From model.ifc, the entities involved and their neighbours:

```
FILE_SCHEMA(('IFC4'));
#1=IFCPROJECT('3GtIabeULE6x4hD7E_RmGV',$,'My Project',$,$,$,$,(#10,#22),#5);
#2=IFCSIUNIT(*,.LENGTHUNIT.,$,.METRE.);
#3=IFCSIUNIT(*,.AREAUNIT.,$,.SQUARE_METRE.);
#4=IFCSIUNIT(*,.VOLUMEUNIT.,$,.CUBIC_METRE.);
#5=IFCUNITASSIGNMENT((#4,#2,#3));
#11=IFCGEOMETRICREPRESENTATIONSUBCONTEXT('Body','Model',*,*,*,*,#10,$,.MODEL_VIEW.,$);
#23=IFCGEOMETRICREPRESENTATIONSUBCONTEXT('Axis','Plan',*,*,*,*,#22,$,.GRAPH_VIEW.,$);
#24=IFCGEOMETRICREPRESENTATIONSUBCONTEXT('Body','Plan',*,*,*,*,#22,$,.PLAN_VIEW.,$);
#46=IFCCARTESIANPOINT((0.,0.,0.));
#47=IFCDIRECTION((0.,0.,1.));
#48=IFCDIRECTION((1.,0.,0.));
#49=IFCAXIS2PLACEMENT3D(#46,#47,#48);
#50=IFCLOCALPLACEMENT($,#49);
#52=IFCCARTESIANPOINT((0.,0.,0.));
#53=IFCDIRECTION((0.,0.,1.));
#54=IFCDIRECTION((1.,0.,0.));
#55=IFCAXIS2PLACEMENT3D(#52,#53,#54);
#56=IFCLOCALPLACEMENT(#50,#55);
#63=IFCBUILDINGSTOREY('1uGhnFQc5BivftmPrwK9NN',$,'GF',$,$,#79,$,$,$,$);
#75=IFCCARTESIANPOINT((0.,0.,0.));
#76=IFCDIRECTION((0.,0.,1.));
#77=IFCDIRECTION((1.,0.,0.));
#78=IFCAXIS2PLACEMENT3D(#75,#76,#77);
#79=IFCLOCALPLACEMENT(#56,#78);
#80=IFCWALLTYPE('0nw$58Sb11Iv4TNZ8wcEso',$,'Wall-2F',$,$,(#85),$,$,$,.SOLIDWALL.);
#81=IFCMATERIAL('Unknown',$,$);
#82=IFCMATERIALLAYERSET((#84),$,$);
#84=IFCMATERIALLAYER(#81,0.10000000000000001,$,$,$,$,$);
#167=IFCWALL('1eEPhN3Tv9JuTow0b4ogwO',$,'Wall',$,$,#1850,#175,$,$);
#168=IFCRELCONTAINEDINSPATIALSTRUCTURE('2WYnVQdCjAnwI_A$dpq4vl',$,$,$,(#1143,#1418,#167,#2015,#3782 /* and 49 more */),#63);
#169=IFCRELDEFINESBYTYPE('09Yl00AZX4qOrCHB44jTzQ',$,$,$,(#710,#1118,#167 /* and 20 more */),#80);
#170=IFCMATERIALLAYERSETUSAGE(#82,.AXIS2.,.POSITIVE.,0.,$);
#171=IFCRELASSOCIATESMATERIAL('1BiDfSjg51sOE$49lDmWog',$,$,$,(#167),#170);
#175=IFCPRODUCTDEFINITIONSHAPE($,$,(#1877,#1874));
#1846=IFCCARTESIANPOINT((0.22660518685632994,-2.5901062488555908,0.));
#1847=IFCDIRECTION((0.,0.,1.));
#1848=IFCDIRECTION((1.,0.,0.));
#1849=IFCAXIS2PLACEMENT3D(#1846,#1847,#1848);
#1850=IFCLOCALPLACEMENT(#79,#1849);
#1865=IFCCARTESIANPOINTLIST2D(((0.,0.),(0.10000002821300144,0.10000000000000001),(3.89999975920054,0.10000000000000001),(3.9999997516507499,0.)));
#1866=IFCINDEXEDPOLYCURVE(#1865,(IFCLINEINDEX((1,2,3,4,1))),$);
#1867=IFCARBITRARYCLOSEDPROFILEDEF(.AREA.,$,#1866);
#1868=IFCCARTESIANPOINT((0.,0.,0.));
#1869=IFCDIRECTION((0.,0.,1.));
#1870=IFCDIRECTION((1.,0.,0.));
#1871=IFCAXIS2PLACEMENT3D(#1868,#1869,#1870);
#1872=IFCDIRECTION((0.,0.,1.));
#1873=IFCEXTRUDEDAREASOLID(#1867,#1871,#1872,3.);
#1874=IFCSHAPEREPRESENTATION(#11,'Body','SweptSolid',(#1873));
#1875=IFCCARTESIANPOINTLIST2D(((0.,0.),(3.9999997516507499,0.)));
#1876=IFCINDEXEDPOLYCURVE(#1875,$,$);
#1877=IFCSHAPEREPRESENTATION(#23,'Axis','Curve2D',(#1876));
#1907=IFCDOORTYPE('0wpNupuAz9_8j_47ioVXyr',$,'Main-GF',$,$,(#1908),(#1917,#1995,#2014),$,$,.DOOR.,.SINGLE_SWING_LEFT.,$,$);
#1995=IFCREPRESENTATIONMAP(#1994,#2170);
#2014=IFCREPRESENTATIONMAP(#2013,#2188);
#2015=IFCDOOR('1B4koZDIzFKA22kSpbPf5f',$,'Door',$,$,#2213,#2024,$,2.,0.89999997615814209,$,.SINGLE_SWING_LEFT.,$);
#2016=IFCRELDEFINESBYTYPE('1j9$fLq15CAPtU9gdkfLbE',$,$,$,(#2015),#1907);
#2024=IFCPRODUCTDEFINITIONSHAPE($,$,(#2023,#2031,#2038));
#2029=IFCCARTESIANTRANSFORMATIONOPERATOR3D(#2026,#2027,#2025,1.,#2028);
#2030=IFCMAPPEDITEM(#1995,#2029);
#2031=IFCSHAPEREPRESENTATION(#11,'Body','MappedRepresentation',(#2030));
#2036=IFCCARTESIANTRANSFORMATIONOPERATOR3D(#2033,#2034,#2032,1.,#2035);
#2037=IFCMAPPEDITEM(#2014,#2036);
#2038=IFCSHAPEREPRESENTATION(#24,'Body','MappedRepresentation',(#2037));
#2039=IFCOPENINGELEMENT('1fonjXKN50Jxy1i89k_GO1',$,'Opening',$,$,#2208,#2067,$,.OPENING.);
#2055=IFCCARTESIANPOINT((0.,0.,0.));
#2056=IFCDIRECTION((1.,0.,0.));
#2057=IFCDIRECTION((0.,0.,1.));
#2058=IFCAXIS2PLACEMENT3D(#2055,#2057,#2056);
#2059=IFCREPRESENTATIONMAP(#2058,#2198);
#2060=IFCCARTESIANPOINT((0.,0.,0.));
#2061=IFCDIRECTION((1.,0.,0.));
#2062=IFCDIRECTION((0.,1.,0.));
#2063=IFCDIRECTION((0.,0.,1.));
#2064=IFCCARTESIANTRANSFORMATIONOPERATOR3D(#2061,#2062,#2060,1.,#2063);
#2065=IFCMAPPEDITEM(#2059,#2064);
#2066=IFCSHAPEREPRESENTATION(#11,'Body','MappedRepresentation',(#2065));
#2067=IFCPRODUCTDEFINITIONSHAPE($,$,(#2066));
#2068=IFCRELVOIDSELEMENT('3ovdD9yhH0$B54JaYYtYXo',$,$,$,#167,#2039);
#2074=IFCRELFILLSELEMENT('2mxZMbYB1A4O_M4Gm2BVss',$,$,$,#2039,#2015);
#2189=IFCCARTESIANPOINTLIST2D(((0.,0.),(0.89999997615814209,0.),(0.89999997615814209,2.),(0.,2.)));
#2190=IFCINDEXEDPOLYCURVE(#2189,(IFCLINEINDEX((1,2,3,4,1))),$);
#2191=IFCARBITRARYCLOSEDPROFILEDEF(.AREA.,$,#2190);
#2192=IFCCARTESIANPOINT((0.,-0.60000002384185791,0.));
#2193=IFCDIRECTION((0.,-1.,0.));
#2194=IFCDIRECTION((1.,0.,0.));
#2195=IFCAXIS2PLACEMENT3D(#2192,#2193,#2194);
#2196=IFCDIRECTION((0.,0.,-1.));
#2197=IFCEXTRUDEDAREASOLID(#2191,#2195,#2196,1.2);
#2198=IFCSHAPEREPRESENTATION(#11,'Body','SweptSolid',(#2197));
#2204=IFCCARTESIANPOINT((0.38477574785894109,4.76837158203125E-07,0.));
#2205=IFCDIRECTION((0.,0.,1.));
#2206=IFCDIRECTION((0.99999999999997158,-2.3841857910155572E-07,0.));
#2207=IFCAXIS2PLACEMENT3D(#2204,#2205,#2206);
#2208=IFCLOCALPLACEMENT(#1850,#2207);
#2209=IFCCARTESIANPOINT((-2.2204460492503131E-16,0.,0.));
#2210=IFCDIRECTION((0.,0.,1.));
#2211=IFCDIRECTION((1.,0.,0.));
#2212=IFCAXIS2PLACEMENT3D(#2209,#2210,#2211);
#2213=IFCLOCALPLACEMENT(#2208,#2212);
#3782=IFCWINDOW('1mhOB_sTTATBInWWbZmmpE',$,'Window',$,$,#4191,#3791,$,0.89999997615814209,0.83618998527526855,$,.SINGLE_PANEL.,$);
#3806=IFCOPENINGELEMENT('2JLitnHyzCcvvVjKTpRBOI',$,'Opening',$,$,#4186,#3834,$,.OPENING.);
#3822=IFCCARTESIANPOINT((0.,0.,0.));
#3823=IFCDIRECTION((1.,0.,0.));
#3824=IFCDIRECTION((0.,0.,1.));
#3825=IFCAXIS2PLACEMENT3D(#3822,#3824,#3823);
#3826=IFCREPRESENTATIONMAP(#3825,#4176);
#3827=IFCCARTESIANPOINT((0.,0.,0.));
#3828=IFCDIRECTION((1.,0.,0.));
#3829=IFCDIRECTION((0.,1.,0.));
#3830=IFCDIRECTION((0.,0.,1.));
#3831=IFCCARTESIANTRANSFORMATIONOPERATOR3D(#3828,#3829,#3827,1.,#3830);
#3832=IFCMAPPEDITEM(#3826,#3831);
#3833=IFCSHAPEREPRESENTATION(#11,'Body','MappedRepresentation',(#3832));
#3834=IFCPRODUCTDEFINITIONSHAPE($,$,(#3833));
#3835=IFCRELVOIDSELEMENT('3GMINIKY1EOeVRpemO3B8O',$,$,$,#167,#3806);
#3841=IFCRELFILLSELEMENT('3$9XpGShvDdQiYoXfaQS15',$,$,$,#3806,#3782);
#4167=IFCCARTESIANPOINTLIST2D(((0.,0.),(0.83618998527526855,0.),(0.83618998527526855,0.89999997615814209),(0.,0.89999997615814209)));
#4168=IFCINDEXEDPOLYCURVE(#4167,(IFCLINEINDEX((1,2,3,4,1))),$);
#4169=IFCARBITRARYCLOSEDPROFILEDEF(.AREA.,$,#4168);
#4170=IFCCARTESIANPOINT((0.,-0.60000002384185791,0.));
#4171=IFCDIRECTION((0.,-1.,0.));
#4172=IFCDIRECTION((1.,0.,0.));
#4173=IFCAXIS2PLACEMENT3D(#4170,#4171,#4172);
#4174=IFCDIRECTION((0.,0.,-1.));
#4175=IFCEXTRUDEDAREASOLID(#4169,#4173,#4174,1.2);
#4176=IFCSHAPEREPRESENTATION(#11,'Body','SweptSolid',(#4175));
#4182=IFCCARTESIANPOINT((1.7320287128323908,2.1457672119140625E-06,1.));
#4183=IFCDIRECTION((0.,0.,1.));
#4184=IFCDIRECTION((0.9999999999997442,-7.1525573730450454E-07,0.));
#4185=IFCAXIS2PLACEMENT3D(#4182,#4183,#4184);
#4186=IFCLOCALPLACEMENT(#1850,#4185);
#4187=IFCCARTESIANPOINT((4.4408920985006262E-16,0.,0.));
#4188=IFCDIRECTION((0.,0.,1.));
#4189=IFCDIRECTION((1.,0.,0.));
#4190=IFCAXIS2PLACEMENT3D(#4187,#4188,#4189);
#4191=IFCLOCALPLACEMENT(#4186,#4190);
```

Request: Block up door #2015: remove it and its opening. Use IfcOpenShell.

```python
import ifcopenshell
import ifcopenshell.api.feature
import ifcopenshell.api.root
import ifcopenshell.geom
import ifcopenshell.util.shape

model = ifcopenshell.open("model.ifc")
settings = ifcopenshell.geom.settings()


def volume(element):
    """Net volume in cubic metres, openings subtracted."""
    shape = ifcopenshell.geom.create_shape(settings, element)
    return ifcopenshell.util.shape.get_volume(shape.geometry)


door = model.by_id(2015)
opening = door.FillsVoids[0].RelatingOpeningElement
wall = opening.VoidsElements[0].RelatingBuildingElement
before = volume(wall)

ifcopenshell.api.root.remove_product(model, product=door)
ifcopenshell.api.feature.remove_feature(model, feature=opening)

after = volume(wall)

print(f"wall volume {before:.3f} -> {after:.3f} m3")

model.write("model-out.ifc")
```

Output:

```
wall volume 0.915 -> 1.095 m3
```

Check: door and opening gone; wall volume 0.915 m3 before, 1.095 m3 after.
